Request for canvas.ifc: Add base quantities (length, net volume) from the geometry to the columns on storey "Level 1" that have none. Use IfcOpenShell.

First a look at what the model holds.

```python
import ifcopenshell
import ifcopenshell.util.element
import ifcopenshell.util.unit

model = ifcopenshell.open("canvas.ifc")
print(model.schema)
for unit_type in ("LENGTHUNIT", "AREAUNIT", "VOLUMEUNIT"):
    print(unit_type, ifcopenshell.util.unit.calculate_unit_scale(model, unit_type))
storey = next(s for s in model.by_type("IfcBuildingStorey") if s.Name == "Level 1")
columns = [e for e in ifcopenshell.util.element.get_decomposition(storey) if e.is_a("IfcColumn")]
for e in sorted(columns, key=lambda e: e.id()):
    print(e.id(), e.is_a(), e.Name, list(ifcopenshell.util.element.get_psets(e, qtos_only=True)), sep=" | ")
```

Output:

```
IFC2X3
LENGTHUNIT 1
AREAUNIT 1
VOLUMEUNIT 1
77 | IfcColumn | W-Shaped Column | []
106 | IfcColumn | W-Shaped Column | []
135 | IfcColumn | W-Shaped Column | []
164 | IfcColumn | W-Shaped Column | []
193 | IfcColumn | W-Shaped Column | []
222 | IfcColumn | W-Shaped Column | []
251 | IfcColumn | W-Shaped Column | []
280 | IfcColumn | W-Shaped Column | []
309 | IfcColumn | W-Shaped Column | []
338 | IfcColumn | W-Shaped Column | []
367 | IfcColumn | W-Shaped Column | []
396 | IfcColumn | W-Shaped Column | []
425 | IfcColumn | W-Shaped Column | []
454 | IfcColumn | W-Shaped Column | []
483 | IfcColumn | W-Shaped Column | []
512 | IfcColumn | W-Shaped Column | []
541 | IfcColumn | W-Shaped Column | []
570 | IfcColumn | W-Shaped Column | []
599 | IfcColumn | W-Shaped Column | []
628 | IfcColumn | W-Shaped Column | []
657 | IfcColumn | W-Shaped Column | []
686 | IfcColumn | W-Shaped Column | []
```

```python
import ifcopenshell
import ifcopenshell.api.pset
import ifcopenshell.geom
import ifcopenshell.util.element
import ifcopenshell.util.shape
import ifcopenshell.util.unit

model = ifcopenshell.open("canvas.ifc")
unit_scale = ifcopenshell.util.unit.calculate_unit_scale(model)
volume_scale = ifcopenshell.util.unit.calculate_unit_scale(model, "VOLUMEUNIT")
settings = ifcopenshell.geom.settings()

storey = next(s for s in model.by_type("IfcBuildingStorey") if s.Name == "Level 1")
columns = [e for e in ifcopenshell.util.element.get_decomposition(storey) if e.is_a("IfcColumn")]

for e in sorted(columns, key=lambda e: e.id()):
    if ifcopenshell.util.element.get_psets(e, qtos_only=True, should_inherit=False):
        continue
    # Geometry comes back in metres, in the element's own axes.
    shape = ifcopenshell.geom.create_shape(settings, e)
    values = {
        "Length": ifcopenshell.util.shape.get_z(shape.geometry) / unit_scale,
        "NetVolume": ifcopenshell.util.shape.get_volume(shape.geometry) / volume_scale,
    }
    qto = ifcopenshell.api.pset.add_qto(model, product=e, name="BaseQuantities")
    ifcopenshell.api.pset.edit_qto(model, qto=qto, properties=values)
    print(e.id(), {k: round(v, 3) for k, v in values.items()})

model.write("canvas_updated.ifc")
```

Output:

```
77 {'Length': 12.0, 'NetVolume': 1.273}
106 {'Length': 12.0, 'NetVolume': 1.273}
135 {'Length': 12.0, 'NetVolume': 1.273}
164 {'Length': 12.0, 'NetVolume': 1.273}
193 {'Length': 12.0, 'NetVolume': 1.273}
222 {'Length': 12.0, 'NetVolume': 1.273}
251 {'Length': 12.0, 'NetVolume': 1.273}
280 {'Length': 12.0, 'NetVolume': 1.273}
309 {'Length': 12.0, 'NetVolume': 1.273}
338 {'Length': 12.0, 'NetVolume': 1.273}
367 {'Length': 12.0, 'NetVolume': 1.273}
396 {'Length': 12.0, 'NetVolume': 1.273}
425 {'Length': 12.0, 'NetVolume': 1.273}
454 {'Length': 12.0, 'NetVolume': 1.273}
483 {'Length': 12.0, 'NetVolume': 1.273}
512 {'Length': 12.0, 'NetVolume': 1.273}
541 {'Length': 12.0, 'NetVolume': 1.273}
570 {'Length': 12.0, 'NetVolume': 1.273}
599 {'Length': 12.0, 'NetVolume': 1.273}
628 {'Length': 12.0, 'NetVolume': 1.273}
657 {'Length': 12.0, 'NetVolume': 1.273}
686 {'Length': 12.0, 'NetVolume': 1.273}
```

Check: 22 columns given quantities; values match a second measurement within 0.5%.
